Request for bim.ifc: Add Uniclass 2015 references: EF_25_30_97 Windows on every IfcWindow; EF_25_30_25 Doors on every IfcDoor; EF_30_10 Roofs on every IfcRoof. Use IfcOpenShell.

First a look at what the model holds.

```python
import ifcopenshell

model = ifcopenshell.open("bim.ifc")
print(model.schema)
print("classifications:", [c.Name for c in model.by_type("IfcClassification")])
for ifc_class in ("IfcDoor", "IfcRoof", "IfcStair", "IfcWall", "IfcWindow"):
    print(ifc_class, len(model.by_type(ifc_class)))
```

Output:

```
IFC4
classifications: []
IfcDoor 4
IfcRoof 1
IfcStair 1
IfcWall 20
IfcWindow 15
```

```python
import ifcopenshell
import ifcopenshell.api.classification

model = ifcopenshell.open("bim.ifc")

system = ifcopenshell.api.classification.add_classification(model, classification="Uniclass 2015")

codes = {
    "IfcWindow": ("EF_25_30_97", "Windows"),
    "IfcDoor": ("EF_25_30_25", "Doors"),
    "IfcRoof": ("EF_30_10", "Roofs"),
}
for ifc_class, (code, name) in codes.items():
    products = model.by_type(ifc_class)
    ifcopenshell.api.classification.add_reference(
        model, products=products, classification=system, identification=code, name=name
    )
    print(code, len(products))

model.write("bim_updated.ifc")
```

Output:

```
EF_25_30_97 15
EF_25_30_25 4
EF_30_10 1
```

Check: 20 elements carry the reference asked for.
